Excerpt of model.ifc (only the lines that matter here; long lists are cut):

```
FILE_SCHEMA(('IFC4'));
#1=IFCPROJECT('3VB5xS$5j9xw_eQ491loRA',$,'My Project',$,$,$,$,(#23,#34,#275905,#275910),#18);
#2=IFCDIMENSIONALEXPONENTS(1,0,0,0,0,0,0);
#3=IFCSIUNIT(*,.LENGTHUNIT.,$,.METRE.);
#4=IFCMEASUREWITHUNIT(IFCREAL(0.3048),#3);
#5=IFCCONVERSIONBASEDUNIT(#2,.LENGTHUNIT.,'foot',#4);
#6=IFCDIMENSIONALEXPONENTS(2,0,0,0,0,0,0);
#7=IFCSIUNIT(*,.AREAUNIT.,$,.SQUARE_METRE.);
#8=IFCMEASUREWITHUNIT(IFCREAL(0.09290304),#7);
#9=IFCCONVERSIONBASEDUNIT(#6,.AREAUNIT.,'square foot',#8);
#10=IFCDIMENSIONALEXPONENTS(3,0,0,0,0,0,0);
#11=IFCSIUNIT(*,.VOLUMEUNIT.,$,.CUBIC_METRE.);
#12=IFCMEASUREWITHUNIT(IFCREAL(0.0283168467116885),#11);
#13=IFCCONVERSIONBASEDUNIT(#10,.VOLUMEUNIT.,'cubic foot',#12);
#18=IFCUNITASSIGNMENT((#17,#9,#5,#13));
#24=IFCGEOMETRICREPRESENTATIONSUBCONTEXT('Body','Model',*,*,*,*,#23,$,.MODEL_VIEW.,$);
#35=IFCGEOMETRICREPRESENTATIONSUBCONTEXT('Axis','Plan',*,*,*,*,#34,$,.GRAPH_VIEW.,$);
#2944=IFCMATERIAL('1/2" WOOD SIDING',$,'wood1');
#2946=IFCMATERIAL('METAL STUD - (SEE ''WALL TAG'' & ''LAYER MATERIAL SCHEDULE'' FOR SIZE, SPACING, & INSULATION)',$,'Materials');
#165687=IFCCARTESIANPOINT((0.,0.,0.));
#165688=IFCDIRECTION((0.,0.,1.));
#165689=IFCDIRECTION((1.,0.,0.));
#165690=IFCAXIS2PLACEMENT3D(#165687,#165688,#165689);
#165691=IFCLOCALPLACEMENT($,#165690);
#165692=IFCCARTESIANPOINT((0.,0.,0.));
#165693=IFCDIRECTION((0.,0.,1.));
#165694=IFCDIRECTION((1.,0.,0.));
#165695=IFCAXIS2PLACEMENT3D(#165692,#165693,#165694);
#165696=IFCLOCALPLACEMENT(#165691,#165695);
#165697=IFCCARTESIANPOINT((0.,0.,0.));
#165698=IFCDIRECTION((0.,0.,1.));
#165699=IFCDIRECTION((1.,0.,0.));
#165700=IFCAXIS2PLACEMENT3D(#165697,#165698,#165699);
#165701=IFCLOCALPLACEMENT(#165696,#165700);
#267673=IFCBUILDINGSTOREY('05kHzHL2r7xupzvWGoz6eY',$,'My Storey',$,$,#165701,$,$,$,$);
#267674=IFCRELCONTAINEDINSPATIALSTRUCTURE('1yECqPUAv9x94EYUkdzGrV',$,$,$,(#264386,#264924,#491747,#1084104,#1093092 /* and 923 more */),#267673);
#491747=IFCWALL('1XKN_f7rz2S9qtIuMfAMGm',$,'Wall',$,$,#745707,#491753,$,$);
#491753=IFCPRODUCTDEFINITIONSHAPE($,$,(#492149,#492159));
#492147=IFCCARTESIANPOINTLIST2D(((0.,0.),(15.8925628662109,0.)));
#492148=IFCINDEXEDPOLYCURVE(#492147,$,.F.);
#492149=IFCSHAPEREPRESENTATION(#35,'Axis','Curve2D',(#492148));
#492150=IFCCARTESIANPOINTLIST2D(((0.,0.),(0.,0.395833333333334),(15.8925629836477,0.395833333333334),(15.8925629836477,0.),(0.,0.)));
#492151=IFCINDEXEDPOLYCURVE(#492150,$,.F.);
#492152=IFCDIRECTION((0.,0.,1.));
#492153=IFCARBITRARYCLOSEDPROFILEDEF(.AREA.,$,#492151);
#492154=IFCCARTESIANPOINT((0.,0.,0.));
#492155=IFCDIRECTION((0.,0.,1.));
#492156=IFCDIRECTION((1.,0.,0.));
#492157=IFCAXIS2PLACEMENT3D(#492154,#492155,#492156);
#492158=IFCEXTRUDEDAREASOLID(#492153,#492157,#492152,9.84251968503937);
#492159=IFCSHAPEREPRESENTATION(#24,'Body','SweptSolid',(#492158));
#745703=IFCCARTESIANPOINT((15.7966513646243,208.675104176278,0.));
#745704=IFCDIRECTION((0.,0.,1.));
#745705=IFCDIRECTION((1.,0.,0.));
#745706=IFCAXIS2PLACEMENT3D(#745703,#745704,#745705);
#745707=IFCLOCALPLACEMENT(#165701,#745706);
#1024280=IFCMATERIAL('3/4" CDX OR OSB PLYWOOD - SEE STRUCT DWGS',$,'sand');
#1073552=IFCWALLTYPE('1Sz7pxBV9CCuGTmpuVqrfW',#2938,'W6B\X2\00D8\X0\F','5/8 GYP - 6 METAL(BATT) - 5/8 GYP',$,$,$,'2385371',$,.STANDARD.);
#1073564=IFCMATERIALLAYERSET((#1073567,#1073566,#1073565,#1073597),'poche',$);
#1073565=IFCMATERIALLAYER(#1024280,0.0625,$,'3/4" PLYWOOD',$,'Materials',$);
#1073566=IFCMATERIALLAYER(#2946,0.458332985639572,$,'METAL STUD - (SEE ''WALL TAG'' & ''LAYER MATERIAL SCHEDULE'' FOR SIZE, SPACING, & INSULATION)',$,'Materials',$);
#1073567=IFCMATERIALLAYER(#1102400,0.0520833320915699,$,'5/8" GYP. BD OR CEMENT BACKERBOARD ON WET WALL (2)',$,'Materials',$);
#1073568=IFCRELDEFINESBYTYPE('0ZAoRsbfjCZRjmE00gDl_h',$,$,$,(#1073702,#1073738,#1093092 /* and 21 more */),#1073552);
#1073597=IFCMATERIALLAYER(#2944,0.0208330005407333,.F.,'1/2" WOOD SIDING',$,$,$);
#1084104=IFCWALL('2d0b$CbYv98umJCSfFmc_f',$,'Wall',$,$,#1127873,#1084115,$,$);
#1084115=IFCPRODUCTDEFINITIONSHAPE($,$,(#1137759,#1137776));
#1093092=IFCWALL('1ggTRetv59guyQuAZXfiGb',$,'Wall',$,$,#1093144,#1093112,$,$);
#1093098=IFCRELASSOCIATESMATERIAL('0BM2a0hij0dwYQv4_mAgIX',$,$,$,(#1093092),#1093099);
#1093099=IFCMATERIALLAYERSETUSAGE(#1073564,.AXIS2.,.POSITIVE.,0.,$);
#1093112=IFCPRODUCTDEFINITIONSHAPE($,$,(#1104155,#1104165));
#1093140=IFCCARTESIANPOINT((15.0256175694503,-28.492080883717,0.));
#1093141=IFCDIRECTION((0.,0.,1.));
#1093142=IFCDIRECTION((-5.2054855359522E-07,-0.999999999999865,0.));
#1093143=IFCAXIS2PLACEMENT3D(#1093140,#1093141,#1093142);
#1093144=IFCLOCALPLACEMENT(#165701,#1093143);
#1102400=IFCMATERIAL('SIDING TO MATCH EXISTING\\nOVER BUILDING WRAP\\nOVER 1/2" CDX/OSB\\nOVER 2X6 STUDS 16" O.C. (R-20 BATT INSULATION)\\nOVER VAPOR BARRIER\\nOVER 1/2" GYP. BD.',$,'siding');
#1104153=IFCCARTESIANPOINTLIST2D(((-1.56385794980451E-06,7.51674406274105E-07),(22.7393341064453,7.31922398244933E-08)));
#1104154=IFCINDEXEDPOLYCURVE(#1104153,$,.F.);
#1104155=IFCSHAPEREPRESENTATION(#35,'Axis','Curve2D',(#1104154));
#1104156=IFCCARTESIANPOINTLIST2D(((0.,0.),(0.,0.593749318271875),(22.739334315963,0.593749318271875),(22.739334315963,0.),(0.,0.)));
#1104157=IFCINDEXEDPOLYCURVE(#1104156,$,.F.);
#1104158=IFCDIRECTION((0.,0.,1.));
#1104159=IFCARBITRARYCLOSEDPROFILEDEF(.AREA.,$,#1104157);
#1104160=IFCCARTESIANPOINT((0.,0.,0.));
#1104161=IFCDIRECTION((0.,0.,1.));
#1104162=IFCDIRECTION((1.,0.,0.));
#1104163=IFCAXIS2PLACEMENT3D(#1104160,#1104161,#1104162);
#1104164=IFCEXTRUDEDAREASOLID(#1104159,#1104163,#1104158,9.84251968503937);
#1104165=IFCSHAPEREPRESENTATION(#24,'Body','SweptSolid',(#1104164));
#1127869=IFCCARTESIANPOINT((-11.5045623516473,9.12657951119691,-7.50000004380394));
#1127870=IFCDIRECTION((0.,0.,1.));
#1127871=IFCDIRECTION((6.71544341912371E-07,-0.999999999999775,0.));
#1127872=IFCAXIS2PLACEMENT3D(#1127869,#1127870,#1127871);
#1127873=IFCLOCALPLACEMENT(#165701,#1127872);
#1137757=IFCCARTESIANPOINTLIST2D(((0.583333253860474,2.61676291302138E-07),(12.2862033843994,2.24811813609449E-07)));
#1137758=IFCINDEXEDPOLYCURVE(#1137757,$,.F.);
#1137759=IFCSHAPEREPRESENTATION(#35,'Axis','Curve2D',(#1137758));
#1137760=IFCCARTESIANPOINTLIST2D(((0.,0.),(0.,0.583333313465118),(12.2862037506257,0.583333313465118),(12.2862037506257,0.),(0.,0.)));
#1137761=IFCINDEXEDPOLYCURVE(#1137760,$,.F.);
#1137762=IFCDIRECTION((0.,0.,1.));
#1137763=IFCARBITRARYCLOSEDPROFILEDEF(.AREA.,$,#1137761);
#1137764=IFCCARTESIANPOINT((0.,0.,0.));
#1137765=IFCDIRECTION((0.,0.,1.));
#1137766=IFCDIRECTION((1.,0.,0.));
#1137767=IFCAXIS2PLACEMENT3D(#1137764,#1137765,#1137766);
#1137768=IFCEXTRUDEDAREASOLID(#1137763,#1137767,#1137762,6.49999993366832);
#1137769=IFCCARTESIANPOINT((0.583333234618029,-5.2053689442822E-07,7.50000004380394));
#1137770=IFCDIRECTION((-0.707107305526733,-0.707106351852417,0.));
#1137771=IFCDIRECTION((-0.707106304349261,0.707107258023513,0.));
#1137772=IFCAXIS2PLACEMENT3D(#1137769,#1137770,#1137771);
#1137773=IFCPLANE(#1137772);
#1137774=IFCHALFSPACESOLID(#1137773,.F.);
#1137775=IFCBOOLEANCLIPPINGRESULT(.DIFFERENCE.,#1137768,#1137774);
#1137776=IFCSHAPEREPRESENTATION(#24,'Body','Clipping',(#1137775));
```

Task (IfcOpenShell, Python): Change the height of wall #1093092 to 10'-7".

```python
import ifcopenshell
import ifcopenshell.geom
import ifcopenshell.util.representation
import ifcopenshell.util.shape
import ifcopenshell.util.unit

model = ifcopenshell.open("model.ifc")
unit_scale = ifcopenshell.util.unit.calculate_unit_scale(model)
settings = ifcopenshell.geom.settings()


def volume(element):
    """Net volume in cubic metres, openings subtracted."""
    shape = ifcopenshell.geom.create_shape(settings, element)
    return ifcopenshell.util.shape.get_volume(shape.geometry)


wall = model.by_guid("1ggTRetv59guyQuAZXfiGb")
before = volume(wall)

body = ifcopenshell.util.representation.get_representation(wall, "Model", "Body")
solid = body.Items[0]
old_height = solid.Depth
solid.Depth = 127 * 0.0254 / unit_scale
after = volume(wall)

print(f"height {old_height:g} -> {solid.Depth:g}, volume {before:.3f} -> {after:.3f} m3")

model.write("model_edited.ifc")
```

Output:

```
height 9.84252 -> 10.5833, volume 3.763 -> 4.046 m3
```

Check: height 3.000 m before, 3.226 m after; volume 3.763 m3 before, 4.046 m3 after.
